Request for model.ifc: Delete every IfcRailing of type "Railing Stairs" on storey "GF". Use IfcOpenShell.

First a look at what the model holds.

```python
import ifcopenshell
import ifcopenshell.util.element

model = ifcopenshell.open("model.ifc")
print(model.schema)
storey = next(s for s in model.by_type("IfcBuildingStorey") if s.Name == "GF")
railings = [e for e in ifcopenshell.util.element.get_decomposition(storey) if e.is_a("IfcRailing")]
seen = {}
for e in railings:
    element_type = ifcopenshell.util.element.get_type(e)
    name = element_type.Name if element_type not in (None, e) else None
    seen[name] = seen.get(name, 0) + 1
for name, count in sorted(seen.items(), key=str):
    print(count, "x", name)
```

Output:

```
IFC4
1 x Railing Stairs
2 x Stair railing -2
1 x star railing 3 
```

```python
import ifcopenshell
import ifcopenshell.api.root
import ifcopenshell.util.element

model = ifcopenshell.open("model.ifc")

storey = next(s for s in model.by_type("IfcBuildingStorey") if s.Name == "GF")
railings = [e for e in ifcopenshell.util.element.get_decomposition(storey) if e.is_a("IfcRailing")]
targets = [e for e in railings if (t := ifcopenshell.util.element.get_type(e)) not in (None, e) and t.Name == "Railing Stairs"]

for e in targets:
    ifcopenshell.api.root.remove_product(model, product=e)
print(len(targets), "removed")

model.write("model_edited.ifc")
```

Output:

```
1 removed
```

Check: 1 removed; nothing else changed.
